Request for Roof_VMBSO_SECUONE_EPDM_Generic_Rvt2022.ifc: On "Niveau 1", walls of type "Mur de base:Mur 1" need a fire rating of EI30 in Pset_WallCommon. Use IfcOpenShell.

First a look at what the model holds.

```python
import ifcopenshell
import ifcopenshell.util.element

model = ifcopenshell.open("Roof_VMBSO_SECUONE_EPDM_Generic_Rvt2022.ifc")
print(model.schema)
storey = next(s for s in model.by_type("IfcBuildingStorey") if s.Name == "Niveau 1")
walls = [e for e in ifcopenshell.util.element.get_decomposition(storey) if e.is_a("IfcWall")]
seen = {}
for e in walls:
    element_type = ifcopenshell.util.element.get_type(e)
    key = (element_type.Name if element_type != e and element_type else None, ifcopenshell.util.element.get_pset(e, "Pset_WallCommon", "FireRating"))
    seen[key] = seen.get(key, 0) + 1
for (name, value), count in sorted(seen.items(), key=str):
    print(count, "x", name, "|", value)
```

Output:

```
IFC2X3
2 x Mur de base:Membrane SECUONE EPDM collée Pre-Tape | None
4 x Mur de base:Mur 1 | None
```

```python
import ifcopenshell
import ifcopenshell.api.pset
import ifcopenshell.util.element

model = ifcopenshell.open("Roof_VMBSO_SECUONE_EPDM_Generic_Rvt2022.ifc")

storey = next(s for s in model.by_type("IfcBuildingStorey") if s.Name == "Niveau 1")
walls = [e for e in ifcopenshell.util.element.get_decomposition(storey) if e.is_a("IfcWall")]

count = 0
for e in walls:
    element_type = ifcopenshell.util.element.get_type(e)
    if element_type in (None, e) or element_type.Name != "Mur de base:Mur 1":
        continue
    # add_pset returns the element's existing set when there is one.
    pset = ifcopenshell.api.pset.add_pset(model, product=e, name="Pset_WallCommon")
    ifcopenshell.api.pset.edit_pset(model, pset=pset, properties={"FireRating": "EI30"})
    count += 1

print(count, "walls updated")

model.write("Roof_VMBSO_SECUONE_EPDM_Generic_Rvt2022_edited.ifc")
```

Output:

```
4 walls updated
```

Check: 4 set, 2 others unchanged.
